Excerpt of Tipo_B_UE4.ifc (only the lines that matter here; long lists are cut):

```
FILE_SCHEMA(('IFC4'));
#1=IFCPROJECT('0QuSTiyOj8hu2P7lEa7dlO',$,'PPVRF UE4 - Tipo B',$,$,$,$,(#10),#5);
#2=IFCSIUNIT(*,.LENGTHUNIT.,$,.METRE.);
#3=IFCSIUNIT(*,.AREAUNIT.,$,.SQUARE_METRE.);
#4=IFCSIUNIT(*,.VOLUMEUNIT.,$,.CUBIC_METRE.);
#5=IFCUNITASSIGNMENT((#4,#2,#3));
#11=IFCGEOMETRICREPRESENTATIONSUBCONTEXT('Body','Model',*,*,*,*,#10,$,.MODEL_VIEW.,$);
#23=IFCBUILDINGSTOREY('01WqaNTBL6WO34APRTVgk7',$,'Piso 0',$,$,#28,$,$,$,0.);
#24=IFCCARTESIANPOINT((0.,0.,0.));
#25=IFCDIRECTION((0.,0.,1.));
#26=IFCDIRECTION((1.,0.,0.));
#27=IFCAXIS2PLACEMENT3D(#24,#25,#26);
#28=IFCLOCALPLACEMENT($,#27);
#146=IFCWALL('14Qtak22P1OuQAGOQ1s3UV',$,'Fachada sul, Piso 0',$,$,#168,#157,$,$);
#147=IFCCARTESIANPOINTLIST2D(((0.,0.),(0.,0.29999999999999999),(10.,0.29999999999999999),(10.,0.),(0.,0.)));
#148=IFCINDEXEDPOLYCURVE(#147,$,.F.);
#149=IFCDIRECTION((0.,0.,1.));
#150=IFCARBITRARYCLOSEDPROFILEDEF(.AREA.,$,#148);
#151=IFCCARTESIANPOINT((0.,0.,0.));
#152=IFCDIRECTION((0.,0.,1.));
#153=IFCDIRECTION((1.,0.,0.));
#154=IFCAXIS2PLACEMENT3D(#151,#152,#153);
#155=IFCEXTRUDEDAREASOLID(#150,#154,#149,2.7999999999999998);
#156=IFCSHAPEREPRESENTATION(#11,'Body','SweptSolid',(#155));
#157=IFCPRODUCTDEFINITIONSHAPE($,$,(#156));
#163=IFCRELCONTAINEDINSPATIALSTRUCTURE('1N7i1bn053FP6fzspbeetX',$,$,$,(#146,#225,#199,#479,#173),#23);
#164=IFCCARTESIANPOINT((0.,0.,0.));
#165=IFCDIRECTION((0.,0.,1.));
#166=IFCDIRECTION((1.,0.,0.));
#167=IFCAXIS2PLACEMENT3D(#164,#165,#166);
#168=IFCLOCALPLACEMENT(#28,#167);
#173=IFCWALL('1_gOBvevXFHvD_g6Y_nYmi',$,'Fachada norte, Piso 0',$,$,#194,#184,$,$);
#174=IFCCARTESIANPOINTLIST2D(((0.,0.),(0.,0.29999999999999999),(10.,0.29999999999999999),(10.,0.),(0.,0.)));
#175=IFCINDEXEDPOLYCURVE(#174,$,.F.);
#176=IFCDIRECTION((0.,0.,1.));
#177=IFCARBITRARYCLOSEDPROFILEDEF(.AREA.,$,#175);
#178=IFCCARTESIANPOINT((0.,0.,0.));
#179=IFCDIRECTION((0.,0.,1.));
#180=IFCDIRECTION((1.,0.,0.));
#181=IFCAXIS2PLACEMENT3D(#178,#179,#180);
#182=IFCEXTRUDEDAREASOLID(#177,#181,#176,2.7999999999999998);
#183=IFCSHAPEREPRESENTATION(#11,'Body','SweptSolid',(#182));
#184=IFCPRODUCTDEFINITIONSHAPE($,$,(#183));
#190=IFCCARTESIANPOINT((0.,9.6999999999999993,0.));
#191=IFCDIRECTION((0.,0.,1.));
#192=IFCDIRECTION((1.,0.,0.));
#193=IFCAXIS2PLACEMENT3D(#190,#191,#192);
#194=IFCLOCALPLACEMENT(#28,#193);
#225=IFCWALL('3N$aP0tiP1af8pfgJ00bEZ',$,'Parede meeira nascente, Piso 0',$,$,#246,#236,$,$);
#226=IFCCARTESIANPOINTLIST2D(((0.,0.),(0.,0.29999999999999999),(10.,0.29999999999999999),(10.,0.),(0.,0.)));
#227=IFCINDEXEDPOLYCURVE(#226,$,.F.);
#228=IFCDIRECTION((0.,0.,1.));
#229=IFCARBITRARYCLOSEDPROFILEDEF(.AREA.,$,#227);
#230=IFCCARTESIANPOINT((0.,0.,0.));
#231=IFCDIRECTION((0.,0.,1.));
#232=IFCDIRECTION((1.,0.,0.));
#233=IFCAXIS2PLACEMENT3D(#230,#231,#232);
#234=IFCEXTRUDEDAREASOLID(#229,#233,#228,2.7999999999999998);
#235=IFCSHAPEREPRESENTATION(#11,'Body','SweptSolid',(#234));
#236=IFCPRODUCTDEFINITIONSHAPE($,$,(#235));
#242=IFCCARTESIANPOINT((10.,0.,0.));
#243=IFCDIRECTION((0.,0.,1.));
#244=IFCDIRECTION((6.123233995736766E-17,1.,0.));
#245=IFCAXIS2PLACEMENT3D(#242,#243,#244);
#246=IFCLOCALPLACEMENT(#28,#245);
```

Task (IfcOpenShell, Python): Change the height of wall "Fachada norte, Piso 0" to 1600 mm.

```python
import ifcopenshell
import ifcopenshell.geom
import ifcopenshell.util.representation
import ifcopenshell.util.shape

model = ifcopenshell.open("Tipo_B_UE4.ifc")
settings = ifcopenshell.geom.settings()


def volume(element):
    """Net volume in cubic metres, openings subtracted."""
    shape = ifcopenshell.geom.create_shape(settings, element)
    return ifcopenshell.util.shape.get_volume(shape.geometry)


wall = model.by_guid("1_gOBvevXFHvD_g6Y_nYmi")
before = volume(wall)

body = ifcopenshell.util.representation.get_representation(wall, "Model", "Body")
solid = body.Items[0]
old_height = solid.Depth
solid.Depth = 1.6
after = volume(wall)

print(f"height {old_height:g} -> {solid.Depth:g}, volume {before:.3f} -> {after:.3f} m3")

model.write("Tipo_B_UE4-out.ifc")
```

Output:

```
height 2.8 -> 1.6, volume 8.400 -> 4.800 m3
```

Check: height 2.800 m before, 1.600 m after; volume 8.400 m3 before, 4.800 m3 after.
